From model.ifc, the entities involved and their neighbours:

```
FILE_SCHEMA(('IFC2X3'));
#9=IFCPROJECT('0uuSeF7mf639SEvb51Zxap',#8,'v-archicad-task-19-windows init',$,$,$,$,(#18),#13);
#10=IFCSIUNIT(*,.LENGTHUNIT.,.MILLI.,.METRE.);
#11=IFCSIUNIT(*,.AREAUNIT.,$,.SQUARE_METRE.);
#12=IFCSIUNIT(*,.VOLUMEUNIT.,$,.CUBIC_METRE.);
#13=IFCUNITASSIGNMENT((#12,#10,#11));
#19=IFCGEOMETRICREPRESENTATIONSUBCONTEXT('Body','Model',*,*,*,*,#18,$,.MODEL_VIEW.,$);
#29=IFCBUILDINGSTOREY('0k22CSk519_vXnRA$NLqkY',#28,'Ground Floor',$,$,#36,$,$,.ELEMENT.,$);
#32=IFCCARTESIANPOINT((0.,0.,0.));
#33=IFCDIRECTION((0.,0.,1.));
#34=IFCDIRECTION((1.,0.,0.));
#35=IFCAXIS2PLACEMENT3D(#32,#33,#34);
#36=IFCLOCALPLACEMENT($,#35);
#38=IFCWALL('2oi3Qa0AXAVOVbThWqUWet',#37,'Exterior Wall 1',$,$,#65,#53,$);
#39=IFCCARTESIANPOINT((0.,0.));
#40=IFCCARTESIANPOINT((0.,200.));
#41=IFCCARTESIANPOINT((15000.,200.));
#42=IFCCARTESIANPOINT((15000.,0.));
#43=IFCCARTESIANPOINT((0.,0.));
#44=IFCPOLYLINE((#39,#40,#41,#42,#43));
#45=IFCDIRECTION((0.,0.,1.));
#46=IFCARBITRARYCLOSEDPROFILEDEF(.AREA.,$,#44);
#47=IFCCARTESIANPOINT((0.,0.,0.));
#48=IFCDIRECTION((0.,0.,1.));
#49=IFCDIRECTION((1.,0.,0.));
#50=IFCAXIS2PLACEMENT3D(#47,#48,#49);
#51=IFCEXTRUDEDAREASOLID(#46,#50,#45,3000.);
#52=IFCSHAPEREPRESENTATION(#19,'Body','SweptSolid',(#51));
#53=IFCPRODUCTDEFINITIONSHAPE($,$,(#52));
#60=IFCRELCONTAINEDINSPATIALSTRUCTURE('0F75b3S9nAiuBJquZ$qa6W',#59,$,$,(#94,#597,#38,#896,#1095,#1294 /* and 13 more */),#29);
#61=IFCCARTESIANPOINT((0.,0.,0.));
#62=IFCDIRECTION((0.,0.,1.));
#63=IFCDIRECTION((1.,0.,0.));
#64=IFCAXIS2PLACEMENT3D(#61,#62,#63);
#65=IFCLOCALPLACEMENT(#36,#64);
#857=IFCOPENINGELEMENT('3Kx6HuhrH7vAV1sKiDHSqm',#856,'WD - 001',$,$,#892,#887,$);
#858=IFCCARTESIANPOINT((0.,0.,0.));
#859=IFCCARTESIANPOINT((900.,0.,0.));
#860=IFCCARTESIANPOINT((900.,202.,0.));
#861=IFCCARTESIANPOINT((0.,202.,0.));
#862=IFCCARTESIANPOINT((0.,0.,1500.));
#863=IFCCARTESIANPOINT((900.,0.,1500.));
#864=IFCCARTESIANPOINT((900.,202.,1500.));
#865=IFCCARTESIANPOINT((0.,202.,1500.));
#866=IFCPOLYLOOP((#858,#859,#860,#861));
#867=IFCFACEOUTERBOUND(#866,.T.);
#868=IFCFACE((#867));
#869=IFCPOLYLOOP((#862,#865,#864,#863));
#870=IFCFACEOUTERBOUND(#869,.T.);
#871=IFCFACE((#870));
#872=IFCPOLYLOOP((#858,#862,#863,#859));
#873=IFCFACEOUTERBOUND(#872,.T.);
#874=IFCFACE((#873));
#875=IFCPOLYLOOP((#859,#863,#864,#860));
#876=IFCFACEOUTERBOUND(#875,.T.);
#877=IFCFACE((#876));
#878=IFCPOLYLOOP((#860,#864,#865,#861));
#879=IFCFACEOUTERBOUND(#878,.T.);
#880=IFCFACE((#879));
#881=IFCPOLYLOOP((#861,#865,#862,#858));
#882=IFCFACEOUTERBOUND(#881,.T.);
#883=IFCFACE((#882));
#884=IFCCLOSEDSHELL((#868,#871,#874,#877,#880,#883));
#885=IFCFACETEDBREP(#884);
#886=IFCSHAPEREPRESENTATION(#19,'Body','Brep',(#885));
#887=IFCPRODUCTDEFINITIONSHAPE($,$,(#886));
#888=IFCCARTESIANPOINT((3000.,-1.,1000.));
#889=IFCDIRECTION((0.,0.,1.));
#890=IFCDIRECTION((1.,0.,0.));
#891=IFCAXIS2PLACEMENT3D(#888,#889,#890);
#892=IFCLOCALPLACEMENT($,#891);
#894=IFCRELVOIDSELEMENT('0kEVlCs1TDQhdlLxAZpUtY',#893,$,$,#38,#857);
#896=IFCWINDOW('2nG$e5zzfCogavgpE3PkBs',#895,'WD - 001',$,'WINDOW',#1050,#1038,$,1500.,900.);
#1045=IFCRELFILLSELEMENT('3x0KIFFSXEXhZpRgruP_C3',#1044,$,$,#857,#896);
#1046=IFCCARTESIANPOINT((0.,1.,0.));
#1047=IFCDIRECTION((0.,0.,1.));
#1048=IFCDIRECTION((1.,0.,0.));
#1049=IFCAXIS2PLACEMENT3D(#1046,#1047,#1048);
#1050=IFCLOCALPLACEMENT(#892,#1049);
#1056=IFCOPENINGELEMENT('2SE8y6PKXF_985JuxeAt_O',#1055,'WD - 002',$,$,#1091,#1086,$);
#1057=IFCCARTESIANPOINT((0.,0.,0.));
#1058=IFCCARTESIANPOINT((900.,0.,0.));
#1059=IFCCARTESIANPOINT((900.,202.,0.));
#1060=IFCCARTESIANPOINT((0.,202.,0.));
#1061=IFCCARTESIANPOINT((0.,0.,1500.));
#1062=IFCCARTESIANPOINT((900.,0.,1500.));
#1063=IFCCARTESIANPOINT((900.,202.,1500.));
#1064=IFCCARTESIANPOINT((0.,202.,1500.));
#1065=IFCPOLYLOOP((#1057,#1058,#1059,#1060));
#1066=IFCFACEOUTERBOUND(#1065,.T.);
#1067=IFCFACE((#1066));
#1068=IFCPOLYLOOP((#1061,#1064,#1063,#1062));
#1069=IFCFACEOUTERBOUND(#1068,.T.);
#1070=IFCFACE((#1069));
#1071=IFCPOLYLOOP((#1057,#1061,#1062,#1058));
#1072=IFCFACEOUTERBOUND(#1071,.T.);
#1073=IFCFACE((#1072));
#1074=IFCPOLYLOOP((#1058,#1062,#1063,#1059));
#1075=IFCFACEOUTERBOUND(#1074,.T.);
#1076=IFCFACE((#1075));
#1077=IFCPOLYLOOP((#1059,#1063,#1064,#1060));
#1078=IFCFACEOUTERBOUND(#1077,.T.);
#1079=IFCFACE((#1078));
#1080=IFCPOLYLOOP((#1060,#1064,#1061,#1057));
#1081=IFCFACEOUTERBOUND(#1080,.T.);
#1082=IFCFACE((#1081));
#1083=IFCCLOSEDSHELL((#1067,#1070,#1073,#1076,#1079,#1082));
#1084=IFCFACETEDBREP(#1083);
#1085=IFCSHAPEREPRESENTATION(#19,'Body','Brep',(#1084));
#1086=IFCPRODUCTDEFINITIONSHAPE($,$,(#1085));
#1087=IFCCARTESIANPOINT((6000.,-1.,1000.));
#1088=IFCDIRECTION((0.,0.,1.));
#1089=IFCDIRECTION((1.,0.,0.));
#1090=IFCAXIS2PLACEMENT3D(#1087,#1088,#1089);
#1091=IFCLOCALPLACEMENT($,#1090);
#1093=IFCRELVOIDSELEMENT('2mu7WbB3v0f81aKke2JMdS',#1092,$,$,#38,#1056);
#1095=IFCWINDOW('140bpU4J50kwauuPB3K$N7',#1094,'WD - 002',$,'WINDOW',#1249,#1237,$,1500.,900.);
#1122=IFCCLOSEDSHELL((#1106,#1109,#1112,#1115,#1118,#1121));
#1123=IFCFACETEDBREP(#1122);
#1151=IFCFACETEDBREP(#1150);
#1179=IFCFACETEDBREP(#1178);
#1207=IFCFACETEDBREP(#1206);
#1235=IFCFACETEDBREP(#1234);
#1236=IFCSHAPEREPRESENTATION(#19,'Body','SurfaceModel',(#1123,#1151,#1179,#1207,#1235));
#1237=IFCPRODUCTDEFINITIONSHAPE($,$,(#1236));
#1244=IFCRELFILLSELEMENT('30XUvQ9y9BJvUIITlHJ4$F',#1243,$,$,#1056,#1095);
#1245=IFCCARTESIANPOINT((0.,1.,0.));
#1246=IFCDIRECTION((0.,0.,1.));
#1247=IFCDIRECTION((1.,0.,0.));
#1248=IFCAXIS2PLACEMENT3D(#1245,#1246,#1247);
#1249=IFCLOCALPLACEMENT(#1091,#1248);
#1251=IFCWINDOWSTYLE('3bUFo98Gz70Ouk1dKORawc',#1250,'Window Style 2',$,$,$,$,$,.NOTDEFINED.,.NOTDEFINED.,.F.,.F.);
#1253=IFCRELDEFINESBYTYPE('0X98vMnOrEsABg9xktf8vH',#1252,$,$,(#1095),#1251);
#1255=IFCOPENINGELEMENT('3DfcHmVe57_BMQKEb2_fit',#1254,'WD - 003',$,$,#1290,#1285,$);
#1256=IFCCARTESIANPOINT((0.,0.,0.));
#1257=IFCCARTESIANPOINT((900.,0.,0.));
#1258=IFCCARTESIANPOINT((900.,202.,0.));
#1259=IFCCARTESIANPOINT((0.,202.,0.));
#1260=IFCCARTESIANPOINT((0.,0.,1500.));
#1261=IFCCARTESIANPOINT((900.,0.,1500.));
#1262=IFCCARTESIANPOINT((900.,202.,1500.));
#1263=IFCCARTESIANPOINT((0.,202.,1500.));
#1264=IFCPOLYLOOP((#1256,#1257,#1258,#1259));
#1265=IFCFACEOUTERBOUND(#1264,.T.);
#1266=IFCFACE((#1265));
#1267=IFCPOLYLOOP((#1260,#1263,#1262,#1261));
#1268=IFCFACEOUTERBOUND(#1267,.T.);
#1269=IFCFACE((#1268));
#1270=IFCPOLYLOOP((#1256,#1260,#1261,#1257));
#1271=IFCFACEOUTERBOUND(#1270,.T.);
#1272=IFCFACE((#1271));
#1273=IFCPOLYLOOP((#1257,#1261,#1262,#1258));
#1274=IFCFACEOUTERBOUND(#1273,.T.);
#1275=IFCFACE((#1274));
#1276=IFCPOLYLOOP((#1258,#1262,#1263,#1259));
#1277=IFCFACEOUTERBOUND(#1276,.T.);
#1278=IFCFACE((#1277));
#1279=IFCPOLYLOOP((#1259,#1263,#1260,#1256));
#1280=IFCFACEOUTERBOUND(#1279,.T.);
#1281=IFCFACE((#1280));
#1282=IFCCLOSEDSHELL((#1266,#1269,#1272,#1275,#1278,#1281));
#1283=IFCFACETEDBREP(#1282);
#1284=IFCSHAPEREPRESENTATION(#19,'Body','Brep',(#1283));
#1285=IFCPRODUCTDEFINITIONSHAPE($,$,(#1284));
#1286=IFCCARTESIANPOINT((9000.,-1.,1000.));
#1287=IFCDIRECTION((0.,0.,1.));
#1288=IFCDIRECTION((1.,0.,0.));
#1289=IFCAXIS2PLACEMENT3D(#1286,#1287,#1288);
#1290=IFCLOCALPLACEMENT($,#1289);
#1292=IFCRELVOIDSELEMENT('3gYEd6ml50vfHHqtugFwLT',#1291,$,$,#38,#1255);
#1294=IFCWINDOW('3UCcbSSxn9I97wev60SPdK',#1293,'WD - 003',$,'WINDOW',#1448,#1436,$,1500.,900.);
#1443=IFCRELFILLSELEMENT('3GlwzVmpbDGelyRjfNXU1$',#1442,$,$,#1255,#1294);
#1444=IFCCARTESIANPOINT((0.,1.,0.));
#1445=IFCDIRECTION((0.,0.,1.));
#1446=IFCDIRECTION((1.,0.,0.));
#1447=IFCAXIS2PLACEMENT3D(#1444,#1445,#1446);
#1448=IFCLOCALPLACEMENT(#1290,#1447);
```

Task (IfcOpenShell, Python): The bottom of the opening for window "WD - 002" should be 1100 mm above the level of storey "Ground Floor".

```python
import numpy as np
import ifcopenshell
import ifcopenshell.api.geometry
import ifcopenshell.geom
import ifcopenshell.util.element
import ifcopenshell.util.placement
import ifcopenshell.util.shape
import ifcopenshell.util.unit

model = ifcopenshell.open("model.ifc")
unit_scale = ifcopenshell.util.unit.calculate_unit_scale(model)

window = model.by_id(1095)
opening = window.FillsVoids[0].RelatingOpeningElement
storey = ifcopenshell.util.element.get_container(window, ifc_class="IfcBuildingStorey")
level = ifcopenshell.util.placement.get_local_placement(storey.ObjectPlacement)[2, 3]

# The opening's origin need not be at the sill, so measure its lowest point.
shape = ifcopenshell.geom.create_shape(ifcopenshell.geom.settings(), opening)
bottom = ifcopenshell.util.shape.get_shape_bottom_elevation(shape, shape.geometry) / unit_scale
dz = level + 1.1 / unit_scale - bottom

shift = np.array([0.0, 0.0, dz])
# The window is placed relative to its opening, so it follows when the opening moves.
matrix = ifcopenshell.util.placement.get_local_placement(opening.ObjectPlacement)
matrix[:3, 3] += shift
ifcopenshell.api.geometry.edit_object_placement(
    model, product=opening, matrix=matrix, is_si=False, should_transform_children=True
)

print(f"moved by {dz * unit_scale:+.3f} m")

model.write("model_edited.ifc")
```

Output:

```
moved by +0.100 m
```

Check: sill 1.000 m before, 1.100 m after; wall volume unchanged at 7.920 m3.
